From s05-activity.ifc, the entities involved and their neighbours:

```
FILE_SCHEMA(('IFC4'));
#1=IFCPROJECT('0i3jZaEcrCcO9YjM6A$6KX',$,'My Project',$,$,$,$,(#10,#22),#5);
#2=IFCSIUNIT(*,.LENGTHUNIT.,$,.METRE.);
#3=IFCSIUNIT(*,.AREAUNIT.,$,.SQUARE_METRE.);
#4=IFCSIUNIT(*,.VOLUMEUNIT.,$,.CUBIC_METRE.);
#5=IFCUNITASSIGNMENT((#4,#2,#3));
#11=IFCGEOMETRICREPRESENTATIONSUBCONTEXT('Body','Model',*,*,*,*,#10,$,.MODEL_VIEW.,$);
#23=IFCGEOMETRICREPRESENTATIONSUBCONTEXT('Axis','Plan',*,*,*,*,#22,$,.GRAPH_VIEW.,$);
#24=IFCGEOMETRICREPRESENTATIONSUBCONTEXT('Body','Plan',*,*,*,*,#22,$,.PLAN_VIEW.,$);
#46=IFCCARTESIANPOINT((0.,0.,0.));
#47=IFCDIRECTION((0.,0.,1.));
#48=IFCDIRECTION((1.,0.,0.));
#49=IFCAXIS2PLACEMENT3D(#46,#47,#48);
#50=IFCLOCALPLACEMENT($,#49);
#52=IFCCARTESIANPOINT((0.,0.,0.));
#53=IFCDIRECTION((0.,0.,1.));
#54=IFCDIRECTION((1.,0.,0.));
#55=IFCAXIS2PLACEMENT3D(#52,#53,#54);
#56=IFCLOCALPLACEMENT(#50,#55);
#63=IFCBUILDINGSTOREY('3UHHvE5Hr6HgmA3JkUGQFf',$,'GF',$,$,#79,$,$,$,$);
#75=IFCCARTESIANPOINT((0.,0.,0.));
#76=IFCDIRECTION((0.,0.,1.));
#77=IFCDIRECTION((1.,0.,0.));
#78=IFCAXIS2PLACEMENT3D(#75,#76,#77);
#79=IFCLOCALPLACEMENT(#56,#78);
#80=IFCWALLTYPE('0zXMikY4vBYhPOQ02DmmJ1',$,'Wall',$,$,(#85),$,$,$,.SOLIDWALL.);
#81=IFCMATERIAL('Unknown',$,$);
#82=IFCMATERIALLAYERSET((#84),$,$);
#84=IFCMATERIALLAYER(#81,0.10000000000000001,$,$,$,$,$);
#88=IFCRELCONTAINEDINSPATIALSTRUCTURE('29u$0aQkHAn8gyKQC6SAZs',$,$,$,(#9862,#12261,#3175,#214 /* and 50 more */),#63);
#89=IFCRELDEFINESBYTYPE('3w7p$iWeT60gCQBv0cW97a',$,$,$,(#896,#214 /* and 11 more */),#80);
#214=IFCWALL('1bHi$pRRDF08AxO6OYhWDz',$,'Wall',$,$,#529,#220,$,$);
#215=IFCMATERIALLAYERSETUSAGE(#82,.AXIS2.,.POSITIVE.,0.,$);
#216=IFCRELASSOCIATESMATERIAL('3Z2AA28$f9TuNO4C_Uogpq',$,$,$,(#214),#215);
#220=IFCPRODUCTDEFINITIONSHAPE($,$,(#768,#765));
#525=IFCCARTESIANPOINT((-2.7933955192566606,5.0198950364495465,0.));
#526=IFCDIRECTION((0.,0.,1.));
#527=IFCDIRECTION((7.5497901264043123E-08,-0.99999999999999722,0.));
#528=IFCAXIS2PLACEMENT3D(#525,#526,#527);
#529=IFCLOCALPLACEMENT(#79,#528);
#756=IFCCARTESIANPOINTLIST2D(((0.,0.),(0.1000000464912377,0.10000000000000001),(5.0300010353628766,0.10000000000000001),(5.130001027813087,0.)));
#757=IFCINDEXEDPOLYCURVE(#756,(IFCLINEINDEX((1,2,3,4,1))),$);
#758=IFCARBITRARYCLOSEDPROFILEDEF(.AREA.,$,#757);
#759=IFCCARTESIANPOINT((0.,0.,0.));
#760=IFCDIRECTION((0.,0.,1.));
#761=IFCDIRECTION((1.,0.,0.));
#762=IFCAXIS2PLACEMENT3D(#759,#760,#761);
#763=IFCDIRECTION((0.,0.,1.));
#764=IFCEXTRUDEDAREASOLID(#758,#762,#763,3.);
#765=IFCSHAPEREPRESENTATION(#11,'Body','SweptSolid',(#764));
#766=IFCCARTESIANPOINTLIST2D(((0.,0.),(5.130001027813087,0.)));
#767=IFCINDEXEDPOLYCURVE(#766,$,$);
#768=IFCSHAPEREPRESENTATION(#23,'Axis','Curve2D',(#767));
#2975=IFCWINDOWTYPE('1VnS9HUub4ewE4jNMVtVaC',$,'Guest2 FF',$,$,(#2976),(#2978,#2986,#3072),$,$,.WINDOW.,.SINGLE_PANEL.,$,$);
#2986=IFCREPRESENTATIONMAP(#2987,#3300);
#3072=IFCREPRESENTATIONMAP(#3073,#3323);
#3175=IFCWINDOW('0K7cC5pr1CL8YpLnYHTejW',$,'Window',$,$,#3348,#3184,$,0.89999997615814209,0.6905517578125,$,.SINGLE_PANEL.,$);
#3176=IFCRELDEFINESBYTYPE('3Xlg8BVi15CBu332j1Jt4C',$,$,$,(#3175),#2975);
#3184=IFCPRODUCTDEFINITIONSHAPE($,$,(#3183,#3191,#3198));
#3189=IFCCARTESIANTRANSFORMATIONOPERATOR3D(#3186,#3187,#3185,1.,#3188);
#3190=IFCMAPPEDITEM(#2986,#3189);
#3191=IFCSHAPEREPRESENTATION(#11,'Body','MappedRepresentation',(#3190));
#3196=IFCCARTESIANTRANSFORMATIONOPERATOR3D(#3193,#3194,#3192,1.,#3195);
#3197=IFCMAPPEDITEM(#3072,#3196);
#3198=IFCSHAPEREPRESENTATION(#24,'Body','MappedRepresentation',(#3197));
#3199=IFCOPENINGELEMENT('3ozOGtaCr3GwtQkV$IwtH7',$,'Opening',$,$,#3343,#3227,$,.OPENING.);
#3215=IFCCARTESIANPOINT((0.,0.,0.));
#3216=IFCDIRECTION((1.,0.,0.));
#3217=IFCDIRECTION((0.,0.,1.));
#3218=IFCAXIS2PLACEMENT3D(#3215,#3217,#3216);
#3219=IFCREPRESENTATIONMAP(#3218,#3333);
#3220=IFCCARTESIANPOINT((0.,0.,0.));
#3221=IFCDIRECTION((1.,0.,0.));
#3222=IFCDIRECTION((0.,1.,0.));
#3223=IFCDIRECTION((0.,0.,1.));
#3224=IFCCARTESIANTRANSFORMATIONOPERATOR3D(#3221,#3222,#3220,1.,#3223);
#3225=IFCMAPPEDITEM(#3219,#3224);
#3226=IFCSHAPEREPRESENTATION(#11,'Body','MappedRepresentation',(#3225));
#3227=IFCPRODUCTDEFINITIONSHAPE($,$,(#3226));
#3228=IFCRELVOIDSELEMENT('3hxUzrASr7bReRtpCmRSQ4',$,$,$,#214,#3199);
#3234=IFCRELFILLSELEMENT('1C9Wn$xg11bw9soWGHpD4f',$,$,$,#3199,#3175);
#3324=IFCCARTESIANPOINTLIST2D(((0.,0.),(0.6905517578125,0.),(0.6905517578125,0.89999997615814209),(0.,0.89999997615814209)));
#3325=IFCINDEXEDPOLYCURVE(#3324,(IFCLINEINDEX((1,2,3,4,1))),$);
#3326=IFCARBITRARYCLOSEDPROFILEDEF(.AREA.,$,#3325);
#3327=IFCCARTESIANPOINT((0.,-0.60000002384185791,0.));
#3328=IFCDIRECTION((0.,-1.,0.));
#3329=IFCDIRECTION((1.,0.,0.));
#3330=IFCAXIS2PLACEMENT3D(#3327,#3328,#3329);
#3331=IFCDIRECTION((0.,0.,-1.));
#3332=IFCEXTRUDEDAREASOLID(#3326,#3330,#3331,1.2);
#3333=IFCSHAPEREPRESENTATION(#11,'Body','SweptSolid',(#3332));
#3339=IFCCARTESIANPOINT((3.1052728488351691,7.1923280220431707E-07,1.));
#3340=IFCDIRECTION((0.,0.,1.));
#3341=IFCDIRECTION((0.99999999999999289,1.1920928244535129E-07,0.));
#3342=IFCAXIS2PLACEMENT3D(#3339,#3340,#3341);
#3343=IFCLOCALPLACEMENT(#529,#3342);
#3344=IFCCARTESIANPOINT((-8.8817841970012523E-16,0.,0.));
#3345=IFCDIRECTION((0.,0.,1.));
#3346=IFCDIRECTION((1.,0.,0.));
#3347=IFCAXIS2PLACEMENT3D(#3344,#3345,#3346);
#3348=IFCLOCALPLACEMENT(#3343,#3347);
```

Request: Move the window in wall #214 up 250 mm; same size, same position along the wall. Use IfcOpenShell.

```python
import numpy as np
import ifcopenshell
import ifcopenshell.api.geometry
import ifcopenshell.util.placement
import ifcopenshell.util.unit

model = ifcopenshell.open("s05-activity.ifc")
unit_scale = ifcopenshell.util.unit.calculate_unit_scale(model)

window = model.by_guid("0K7cC5pr1CL8YpLnYHTejW")
opening = window.FillsVoids[0].RelatingOpeningElement
dz = 0.25 / unit_scale

shift = np.array([0.0, 0.0, dz])
# The window is placed relative to its opening, so it follows when the opening moves.
matrix = ifcopenshell.util.placement.get_local_placement(opening.ObjectPlacement)
matrix[:3, 3] += shift
ifcopenshell.api.geometry.edit_object_placement(
    model, product=opening, matrix=matrix, is_si=False, should_transform_children=True
)

print(f"moved by {dz * unit_scale:+.3f} m")

model.write("s05-activity_rev.ifc")
```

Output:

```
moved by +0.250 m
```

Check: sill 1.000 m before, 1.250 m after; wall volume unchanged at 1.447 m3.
